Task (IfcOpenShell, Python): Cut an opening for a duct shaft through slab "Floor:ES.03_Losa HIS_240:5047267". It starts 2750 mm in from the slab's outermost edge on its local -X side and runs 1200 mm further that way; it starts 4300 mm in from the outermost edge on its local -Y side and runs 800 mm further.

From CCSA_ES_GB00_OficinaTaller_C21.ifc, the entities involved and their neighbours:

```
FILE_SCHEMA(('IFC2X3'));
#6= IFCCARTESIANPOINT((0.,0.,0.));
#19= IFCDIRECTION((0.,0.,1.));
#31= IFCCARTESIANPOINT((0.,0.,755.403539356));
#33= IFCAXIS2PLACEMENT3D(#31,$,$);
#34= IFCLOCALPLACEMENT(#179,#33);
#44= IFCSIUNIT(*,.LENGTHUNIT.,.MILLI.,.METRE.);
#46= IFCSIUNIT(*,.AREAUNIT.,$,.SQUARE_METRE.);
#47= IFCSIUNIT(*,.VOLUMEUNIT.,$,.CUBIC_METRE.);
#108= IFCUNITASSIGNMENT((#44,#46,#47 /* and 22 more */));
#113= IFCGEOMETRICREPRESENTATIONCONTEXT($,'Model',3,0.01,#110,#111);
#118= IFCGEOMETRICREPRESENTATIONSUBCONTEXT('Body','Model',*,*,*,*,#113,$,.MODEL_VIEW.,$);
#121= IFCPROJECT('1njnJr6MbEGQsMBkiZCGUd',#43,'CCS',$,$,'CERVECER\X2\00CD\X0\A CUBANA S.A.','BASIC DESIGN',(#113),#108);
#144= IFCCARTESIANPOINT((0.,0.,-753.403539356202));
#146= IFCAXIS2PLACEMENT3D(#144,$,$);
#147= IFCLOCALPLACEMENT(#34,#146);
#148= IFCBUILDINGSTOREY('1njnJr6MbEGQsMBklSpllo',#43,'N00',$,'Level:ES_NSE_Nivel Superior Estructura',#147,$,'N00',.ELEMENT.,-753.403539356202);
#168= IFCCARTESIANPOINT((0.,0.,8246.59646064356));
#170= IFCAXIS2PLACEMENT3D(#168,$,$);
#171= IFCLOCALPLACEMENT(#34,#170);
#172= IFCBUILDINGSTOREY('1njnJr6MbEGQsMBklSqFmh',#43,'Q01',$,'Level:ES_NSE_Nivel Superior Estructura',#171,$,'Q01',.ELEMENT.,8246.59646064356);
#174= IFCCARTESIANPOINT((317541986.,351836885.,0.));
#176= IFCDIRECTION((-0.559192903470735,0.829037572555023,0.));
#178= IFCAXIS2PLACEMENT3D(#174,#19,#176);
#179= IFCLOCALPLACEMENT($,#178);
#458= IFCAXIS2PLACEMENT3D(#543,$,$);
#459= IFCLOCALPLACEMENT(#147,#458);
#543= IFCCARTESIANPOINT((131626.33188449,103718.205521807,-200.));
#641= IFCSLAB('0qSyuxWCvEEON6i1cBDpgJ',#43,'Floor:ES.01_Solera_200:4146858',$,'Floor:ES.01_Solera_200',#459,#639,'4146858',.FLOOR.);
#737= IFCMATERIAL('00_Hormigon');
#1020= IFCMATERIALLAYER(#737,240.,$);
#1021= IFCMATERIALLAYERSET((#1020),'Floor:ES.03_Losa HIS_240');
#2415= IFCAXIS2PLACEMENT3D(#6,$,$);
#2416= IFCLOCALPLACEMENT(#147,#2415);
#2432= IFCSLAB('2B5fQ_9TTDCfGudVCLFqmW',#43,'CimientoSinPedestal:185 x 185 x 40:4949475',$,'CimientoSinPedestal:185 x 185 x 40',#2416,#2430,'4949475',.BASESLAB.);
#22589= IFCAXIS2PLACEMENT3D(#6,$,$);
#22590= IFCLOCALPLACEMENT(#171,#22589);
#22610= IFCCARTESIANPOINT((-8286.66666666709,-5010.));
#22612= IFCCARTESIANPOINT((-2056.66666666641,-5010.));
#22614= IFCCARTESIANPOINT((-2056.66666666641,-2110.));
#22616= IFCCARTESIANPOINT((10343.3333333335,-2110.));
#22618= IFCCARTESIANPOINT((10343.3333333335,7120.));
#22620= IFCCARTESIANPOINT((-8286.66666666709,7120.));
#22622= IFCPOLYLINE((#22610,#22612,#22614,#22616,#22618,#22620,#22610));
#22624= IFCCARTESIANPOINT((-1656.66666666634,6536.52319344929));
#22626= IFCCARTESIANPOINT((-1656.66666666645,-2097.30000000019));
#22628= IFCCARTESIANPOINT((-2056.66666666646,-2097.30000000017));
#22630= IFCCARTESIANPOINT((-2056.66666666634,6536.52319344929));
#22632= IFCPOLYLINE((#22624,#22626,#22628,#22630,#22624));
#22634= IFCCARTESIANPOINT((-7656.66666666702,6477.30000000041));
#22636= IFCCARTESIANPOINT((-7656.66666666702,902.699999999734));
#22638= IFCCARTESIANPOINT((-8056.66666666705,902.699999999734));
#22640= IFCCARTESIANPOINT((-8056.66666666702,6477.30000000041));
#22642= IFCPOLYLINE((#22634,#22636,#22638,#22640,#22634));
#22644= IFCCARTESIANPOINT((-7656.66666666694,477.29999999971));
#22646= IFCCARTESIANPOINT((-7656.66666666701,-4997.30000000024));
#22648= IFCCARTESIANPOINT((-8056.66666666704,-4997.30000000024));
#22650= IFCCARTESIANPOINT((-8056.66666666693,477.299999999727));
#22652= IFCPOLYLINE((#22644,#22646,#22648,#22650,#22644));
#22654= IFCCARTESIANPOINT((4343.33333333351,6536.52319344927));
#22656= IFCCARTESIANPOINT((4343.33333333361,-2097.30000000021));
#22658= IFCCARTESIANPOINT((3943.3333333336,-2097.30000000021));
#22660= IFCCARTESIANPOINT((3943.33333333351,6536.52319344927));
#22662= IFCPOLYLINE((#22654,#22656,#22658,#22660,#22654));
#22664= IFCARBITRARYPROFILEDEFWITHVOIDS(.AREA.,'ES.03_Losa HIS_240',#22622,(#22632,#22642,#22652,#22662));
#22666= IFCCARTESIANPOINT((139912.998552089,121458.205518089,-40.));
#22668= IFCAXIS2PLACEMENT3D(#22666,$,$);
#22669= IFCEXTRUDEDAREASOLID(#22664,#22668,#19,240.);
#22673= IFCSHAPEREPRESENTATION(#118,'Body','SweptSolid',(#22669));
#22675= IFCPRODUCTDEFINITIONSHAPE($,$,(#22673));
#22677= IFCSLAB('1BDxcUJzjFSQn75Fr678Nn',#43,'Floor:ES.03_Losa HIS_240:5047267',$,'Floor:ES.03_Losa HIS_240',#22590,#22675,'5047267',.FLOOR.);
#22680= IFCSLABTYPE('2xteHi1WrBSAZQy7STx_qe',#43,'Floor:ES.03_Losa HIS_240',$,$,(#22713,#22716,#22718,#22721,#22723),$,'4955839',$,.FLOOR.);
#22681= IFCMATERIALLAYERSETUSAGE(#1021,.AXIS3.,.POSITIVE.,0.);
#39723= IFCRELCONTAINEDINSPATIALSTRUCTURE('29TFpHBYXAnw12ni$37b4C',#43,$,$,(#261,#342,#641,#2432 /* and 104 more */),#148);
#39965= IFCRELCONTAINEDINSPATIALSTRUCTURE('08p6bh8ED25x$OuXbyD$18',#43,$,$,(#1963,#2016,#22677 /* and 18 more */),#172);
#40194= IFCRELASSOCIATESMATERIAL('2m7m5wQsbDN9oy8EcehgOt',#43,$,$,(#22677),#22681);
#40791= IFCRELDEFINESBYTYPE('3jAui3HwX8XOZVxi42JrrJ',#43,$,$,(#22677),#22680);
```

```python
import numpy as np
import ifcopenshell
import ifcopenshell.api.feature
import ifcopenshell.api.geometry
import ifcopenshell.api.root
import ifcopenshell.geom
import ifcopenshell.util.placement
import ifcopenshell.util.representation
import ifcopenshell.util.shape
import ifcopenshell.util.unit

model = ifcopenshell.open("CCSA_ES_GB00_OficinaTaller_C21.ifc")
unit_scale = ifcopenshell.util.unit.calculate_unit_scale(model)
settings = ifcopenshell.geom.settings()


def volume(element):
    """Net volume in cubic metres, openings subtracted."""
    shape = ifcopenshell.geom.create_shape(settings, element)
    return ifcopenshell.util.shape.get_volume(shape.geometry)


slab = model.by_guid("1BDxcUJzjFSQn75Fr678Nn")
before = volume(slab)

# Extent in the slab's own axes, in metres. The edges named are its -X and -Y sides.
slab_shape = ifcopenshell.geom.create_shape(settings, slab)
vertices = ifcopenshell.util.shape.get_vertices(slab_shape.geometry)
x_min, y_min, bottom = vertices.min(axis=0)
top = vertices[:, 2].max()

opening = ifcopenshell.api.root.create_entity(model, ifc_class="IfcOpeningElement", name="Duct shaft opening")
context = ifcopenshell.util.representation.get_context(model, "Model", "Body", "MODEL_VIEW")
width, depth = 1.2, 0.8
outline = [(0.0, 0.0), (width, 0.0), (width, depth), (0.0, depth), (0.0, 0.0)]
# Overshoot both faces by 50 mm so the cut is clean.
shape = ifcopenshell.api.geometry.add_slab_representation(
    model, context=context, depth=top - bottom + 0.1, polyline=outline
)
ifcopenshell.api.geometry.assign_representation(model, product=opening, representation=shape)

matrix = ifcopenshell.util.placement.get_local_placement(slab.ObjectPlacement)
matrix[:, 3] = matrix @ np.append(np.array([x_min + 2.75, y_min + 4.3, bottom - 0.05]) / unit_scale, 1.0)
ifcopenshell.api.geometry.edit_object_placement(model, product=opening, matrix=matrix, is_si=False)
ifcopenshell.api.feature.add_feature(model, feature=opening, element=slab)

after = volume(slab)

print(f"slab volume {before:.3f} -> {after:.3f} m3")

model.write("CCSA_ES_GB00_OficinaTaller_C21_edited.ifc")
```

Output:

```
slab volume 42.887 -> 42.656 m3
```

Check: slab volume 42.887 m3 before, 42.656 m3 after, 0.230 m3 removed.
